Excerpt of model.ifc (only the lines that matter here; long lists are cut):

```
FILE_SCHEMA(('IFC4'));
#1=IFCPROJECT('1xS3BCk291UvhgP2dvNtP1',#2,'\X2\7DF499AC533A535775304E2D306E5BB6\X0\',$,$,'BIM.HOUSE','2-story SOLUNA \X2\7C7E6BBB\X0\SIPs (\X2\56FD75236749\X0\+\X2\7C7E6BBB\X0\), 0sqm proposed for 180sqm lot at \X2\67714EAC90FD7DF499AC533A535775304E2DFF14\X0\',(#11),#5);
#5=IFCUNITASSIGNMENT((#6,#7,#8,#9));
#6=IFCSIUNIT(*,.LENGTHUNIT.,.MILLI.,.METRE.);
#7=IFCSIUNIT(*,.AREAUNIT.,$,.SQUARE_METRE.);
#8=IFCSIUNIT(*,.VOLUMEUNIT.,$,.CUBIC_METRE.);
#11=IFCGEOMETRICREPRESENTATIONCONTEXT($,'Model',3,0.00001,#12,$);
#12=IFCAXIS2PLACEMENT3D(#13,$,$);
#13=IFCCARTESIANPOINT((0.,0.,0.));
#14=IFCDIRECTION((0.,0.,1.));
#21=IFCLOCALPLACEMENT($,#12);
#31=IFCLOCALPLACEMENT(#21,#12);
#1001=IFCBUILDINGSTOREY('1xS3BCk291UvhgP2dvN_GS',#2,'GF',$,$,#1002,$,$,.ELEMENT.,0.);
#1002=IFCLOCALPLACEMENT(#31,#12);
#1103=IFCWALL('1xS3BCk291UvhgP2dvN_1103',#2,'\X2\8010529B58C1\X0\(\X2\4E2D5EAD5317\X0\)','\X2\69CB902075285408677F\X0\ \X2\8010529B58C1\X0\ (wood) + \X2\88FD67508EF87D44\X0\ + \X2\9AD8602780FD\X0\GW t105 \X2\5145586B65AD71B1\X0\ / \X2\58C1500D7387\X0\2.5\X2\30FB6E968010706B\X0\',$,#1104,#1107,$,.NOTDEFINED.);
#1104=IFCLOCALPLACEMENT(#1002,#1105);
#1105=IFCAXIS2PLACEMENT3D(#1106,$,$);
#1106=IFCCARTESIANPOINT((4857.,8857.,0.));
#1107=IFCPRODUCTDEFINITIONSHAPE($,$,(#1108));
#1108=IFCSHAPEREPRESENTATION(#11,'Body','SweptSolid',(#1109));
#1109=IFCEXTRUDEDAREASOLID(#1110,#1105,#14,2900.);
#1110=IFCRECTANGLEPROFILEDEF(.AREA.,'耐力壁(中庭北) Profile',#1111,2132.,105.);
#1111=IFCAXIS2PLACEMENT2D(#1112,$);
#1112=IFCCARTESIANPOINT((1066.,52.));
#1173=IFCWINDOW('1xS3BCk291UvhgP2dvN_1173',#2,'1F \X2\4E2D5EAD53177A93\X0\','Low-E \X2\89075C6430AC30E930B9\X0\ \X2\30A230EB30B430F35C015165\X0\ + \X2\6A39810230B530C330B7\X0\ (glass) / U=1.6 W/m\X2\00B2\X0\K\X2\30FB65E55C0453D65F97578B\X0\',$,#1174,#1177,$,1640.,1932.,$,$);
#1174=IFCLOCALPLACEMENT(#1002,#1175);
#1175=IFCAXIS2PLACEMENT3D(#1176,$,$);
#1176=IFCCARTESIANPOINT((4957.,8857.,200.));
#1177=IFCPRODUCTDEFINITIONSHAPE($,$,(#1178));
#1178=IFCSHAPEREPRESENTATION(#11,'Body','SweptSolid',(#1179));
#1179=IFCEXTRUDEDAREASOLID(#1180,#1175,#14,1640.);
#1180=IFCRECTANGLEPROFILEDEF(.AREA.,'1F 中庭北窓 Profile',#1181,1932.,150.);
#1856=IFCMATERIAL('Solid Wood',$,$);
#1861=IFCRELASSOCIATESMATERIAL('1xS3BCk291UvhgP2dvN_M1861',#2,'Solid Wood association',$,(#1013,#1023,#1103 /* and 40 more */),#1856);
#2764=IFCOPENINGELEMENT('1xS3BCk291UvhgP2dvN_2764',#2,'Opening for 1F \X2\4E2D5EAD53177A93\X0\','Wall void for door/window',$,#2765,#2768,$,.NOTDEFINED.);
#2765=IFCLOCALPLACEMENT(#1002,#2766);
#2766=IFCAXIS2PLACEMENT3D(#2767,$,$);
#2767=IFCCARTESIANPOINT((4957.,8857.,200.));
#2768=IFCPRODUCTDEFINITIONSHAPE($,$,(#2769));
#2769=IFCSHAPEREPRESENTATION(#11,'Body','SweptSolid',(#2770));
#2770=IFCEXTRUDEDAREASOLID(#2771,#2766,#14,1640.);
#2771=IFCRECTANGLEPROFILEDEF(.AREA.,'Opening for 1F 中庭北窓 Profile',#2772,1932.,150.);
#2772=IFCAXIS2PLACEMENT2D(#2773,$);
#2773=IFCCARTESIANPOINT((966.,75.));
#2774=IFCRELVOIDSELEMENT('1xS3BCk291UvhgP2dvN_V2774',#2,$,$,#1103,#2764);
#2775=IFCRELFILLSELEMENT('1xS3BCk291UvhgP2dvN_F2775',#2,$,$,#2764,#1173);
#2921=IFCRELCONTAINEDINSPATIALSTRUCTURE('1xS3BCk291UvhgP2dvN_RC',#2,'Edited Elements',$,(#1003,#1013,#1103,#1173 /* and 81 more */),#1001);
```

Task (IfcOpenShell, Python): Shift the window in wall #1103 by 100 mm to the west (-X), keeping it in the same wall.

```python
import ifcopenshell
import ifcopenshell.api.geometry
import ifcopenshell.util.placement

model = ifcopenshell.open("model.ifc")

window = model.by_guid("1xS3BCk291UvhgP2dvN_1173")
opening = window.FillsVoids[0].RelatingOpeningElement
wall = opening.VoidsElements[0].RelatingBuildingElement

wall_matrix = ifcopenshell.util.placement.get_local_placement(wall.ObjectPlacement)
shift = wall_matrix[:3, 0] * -100.0
before = ifcopenshell.util.placement.get_local_placement(window.ObjectPlacement)[:3, 3].copy()

# The window is not placed relative to its opening, so move both.
for product in (opening, window):
    matrix = ifcopenshell.util.placement.get_local_placement(product.ObjectPlacement)
    matrix[:3, 3] += shift
    ifcopenshell.api.geometry.edit_object_placement(model, product=product, matrix=matrix, is_si=False)

after = ifcopenshell.util.placement.get_local_placement(window.ObjectPlacement)[:3, 3]
print("window moved by", (after - before).round(3) + 0.0)

model.write("model_updated.ifc")
```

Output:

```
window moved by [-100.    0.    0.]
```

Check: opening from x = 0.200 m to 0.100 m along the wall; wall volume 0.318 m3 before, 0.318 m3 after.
